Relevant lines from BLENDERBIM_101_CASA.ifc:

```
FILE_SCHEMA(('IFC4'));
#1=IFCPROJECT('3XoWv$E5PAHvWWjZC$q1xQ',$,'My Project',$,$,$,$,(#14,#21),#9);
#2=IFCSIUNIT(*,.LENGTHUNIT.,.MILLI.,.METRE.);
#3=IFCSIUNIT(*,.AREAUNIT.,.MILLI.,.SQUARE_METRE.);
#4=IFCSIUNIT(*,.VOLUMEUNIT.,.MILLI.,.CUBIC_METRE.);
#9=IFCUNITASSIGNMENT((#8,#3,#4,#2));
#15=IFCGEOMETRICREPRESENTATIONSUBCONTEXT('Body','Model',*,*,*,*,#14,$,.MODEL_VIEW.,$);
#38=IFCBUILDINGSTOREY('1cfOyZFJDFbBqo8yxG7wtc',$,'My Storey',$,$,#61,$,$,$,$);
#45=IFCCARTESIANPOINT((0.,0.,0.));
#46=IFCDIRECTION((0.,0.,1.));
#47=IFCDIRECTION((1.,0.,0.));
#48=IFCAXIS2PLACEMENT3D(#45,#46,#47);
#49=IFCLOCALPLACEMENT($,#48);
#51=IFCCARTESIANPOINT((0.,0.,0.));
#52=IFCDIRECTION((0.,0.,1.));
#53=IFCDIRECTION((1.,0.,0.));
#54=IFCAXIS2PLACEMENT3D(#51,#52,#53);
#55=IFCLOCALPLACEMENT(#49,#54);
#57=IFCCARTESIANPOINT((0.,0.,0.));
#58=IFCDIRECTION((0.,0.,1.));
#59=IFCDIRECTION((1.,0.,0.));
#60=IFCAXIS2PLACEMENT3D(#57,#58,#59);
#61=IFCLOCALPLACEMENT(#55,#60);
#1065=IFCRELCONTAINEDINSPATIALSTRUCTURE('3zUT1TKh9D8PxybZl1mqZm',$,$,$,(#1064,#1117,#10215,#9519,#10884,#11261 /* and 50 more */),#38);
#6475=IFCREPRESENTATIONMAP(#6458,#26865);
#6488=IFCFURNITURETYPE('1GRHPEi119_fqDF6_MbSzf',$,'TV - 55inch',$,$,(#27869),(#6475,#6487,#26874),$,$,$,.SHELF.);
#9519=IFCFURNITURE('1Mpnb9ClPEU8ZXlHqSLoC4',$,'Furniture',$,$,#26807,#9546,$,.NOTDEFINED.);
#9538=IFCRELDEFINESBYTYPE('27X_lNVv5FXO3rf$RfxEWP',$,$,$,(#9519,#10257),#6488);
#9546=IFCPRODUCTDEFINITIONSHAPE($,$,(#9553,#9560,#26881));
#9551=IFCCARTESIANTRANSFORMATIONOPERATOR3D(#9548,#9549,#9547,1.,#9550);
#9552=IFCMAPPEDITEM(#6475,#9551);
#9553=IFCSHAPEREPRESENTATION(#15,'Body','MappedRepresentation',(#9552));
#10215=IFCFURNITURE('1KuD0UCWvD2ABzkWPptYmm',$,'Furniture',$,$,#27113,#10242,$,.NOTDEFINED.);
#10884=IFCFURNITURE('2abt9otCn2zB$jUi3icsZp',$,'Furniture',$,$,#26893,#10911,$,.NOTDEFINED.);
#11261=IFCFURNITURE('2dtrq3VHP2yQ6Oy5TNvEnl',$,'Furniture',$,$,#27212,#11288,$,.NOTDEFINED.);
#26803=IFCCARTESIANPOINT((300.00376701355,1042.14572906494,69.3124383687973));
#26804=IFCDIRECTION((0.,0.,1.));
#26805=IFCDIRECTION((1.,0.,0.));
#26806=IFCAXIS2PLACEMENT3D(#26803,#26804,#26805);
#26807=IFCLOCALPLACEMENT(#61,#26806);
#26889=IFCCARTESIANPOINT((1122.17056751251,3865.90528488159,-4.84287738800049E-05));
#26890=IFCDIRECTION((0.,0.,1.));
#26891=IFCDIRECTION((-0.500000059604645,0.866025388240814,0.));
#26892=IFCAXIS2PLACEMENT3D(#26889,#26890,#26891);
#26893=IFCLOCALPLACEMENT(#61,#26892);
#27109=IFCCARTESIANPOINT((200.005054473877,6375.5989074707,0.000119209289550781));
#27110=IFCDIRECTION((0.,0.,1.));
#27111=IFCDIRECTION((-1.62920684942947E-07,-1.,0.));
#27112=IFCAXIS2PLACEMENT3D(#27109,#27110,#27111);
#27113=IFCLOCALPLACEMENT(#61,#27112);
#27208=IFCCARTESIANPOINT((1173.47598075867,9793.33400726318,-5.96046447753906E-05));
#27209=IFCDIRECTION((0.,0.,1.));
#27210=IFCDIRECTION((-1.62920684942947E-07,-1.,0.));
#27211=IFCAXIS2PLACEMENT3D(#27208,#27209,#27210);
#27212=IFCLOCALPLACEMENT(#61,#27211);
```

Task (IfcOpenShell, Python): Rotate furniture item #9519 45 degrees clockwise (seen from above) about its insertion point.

```python
import ifcopenshell
import ifcopenshell.api.geometry
import ifcopenshell.util.placement

model = ifcopenshell.open("BLENDERBIM_101_CASA.ifc")

item = model.by_guid("1Mpnb9ClPEU8ZXlHqSLoC4")
matrix = ifcopenshell.util.placement.get_local_placement(item.ObjectPlacement)
matrix = matrix @ ifcopenshell.util.placement.rotation(-45, "Z")
ifcopenshell.api.geometry.edit_object_placement(model, product=item, matrix=matrix, is_si=False)

print(ifcopenshell.util.placement.get_local_placement(item.ObjectPlacement).round(3) + 0.0)

model.write("BLENDERBIM_101_CASA_edited.ifc")
```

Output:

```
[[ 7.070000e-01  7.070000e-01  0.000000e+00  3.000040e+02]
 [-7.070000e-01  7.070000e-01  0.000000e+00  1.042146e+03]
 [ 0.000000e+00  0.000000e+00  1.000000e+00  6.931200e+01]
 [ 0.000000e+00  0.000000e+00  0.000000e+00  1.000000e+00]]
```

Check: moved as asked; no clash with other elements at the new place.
